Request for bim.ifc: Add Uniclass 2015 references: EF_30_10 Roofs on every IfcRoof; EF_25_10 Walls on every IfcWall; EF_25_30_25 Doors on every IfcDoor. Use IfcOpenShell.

First a look at what the model holds.

```python
import ifcopenshell

model = ifcopenshell.open("bim.ifc")
print(model.schema)
print("classifications:", [c.Name for c in model.by_type("IfcClassification")])
for ifc_class in ("IfcDoor", "IfcRoof", "IfcStair", "IfcWall", "IfcWindow"):
    print(ifc_class, len(model.by_type(ifc_class)))
```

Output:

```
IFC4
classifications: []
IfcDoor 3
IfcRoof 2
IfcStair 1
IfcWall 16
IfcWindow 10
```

```python
import ifcopenshell
import ifcopenshell.api.classification

model = ifcopenshell.open("bim.ifc")

system = ifcopenshell.api.classification.add_classification(model, classification="Uniclass 2015")

codes = {
    "IfcRoof": ("EF_30_10", "Roofs"),
    "IfcWall": ("EF_25_10", "Walls"),
    "IfcDoor": ("EF_25_30_25", "Doors"),
}
for ifc_class, (code, name) in codes.items():
    products = model.by_type(ifc_class)
    ifcopenshell.api.classification.add_reference(
        model, products=products, classification=system, identification=code, name=name
    )
    print(code, len(products))

model.write("bim-out.ifc")
```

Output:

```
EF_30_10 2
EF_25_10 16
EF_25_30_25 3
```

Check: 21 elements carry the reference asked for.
